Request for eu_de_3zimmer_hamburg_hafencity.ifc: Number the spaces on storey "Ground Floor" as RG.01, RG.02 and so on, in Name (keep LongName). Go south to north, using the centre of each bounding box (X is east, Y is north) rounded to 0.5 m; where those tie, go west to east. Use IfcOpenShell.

First a look at what the model holds.

```python
import ifcopenshell
import ifcopenshell.util.element
import ifcopenshell.util.placement

model = ifcopenshell.open("eu_de_3zimmer_hamburg_hafencity.ifc")
print(model.schema)
storey = next(s for s in model.by_type("IfcBuildingStorey") if s.Name == "Ground Floor")
spaces = [e for e in ifcopenshell.util.element.get_decomposition(storey) if e.is_a("IfcSpace")]
for e in sorted(spaces, key=lambda e: e.id()):
    origin = ifcopenshell.util.placement.get_local_placement(e.ObjectPlacement)[:3, 3]
    print(e.id(), e.Name, e.LongName, origin.round(2) + 0.0, sep=" | ")
```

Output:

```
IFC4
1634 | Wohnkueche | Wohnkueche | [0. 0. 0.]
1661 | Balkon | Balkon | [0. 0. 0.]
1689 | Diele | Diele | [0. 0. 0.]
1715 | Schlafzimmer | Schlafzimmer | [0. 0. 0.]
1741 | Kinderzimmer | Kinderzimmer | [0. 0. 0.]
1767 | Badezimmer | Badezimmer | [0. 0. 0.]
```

```python
import ifcopenshell
import ifcopenshell.geom
import ifcopenshell.util.element
import ifcopenshell.util.shape

model = ifcopenshell.open("eu_de_3zimmer_hamburg_hafencity.ifc")
settings = ifcopenshell.geom.settings()
settings.set("use-world-coords", True)


def centre(element):
    shape = ifcopenshell.geom.create_shape(settings, element)
    return ifcopenshell.util.shape.get_bbox_centroid(shape.geometry)


storey = next(s for s in model.by_type("IfcBuildingStorey") if s.Name == "Ground Floor")
spaces = [e for e in ifcopenshell.util.element.get_decomposition(storey) if e.is_a("IfcSpace")]

# Insertion points can sit at a corner or the storey origin, so sort by the geometry (in metres).
centres = {e: centre(e) for e in spaces}
spaces.sort(key=lambda e: (round(centres[e][1] / 0.5), centres[e][0]))

for i, e in enumerate(spaces, start=1):
    number = f"RG.{i:02d}"
    e.Name = number
    print(e.id(), number)

model.write("eu_de_3zimmer_hamburg_hafencity_edited.ifc")
```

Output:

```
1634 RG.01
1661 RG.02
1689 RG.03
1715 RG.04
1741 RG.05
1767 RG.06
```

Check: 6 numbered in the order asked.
